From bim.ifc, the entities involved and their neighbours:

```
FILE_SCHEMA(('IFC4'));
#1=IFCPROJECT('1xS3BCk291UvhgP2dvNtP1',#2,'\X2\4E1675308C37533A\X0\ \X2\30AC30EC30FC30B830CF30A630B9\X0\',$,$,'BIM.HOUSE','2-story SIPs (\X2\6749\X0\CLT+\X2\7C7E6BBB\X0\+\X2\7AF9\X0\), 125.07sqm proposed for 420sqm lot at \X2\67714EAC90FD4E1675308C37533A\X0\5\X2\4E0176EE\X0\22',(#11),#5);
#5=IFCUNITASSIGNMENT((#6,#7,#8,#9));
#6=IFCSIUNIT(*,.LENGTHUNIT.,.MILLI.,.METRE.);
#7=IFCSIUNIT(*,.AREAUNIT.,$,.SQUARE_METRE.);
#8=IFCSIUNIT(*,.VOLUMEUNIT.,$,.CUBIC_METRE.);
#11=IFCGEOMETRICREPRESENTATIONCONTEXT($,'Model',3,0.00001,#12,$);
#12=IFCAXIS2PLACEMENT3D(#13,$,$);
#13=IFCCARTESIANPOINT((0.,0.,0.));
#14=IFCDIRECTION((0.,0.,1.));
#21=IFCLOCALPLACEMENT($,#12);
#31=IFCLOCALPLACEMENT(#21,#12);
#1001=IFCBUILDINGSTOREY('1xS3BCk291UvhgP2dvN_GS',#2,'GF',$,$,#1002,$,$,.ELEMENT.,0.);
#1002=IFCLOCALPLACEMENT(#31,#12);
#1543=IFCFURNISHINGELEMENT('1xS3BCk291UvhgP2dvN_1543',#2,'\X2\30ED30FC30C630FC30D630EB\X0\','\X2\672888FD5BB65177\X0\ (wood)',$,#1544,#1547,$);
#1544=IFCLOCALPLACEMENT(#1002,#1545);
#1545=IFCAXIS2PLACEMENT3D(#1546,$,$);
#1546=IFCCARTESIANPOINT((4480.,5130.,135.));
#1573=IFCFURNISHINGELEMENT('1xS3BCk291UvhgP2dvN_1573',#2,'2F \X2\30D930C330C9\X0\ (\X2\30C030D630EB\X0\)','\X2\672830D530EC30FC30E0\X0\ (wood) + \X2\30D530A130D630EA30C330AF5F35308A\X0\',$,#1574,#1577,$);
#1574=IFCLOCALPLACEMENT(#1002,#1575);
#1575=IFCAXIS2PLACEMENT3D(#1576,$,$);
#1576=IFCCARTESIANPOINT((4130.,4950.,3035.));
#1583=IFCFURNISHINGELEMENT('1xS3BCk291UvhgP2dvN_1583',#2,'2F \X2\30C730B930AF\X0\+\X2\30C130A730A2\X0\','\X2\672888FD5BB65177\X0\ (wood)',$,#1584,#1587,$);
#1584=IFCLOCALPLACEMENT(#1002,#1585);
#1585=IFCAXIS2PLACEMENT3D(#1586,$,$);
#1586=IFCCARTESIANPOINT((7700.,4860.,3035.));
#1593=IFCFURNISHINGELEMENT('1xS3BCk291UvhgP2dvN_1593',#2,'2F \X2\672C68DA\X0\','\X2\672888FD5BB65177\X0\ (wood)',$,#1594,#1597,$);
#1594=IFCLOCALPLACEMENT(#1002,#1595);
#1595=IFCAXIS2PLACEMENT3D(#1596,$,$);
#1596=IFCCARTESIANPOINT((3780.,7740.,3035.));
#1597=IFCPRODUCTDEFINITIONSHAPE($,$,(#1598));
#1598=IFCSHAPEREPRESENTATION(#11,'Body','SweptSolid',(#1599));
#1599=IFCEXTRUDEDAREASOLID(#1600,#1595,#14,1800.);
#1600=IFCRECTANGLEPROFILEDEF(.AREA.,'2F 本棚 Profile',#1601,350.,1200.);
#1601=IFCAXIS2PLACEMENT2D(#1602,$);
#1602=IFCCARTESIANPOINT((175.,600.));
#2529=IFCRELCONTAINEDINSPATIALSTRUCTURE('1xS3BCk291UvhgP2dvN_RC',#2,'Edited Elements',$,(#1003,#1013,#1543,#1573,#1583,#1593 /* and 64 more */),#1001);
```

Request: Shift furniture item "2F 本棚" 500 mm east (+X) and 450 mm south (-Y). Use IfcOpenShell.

```python
import ifcopenshell
import ifcopenshell.api.geometry
import ifcopenshell.util.placement
import ifcopenshell.util.unit

model = ifcopenshell.open("bim.ifc")
unit_scale = ifcopenshell.util.unit.calculate_unit_scale(model)

item = model.by_guid("1xS3BCk291UvhgP2dvN_1593")
matrix = ifcopenshell.util.placement.get_local_placement(item.ObjectPlacement)
matrix[0, 3] += 0.5 / unit_scale
matrix[1, 3] -= 0.45 / unit_scale
ifcopenshell.api.geometry.edit_object_placement(model, product=item, matrix=matrix, is_si=False)

print(ifcopenshell.util.placement.get_local_placement(item.ObjectPlacement).round(3) + 0.0)

model.write("bim_v2.ifc")
```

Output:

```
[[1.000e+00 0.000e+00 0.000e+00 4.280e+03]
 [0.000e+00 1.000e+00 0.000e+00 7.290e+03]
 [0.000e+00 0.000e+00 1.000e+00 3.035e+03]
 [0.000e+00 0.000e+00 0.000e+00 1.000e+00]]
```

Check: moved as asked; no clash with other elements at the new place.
